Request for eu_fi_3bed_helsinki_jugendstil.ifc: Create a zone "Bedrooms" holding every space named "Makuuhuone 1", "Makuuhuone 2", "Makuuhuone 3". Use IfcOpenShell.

First a look at what the model holds.

```python
import ifcopenshell

model = ifcopenshell.open("eu_fi_3bed_helsinki_jugendstil.ifc")
print(model.schema)
seen = {}
for space in model.by_type("IfcSpace"):
    seen[space.LongName] = seen.get(space.LongName, 0) + 1
for name, count in sorted(seen.items(), key=str):
    print(count, "x", name)
print("zones:", [z.Name for z in model.by_type("IfcZone")][:20])
```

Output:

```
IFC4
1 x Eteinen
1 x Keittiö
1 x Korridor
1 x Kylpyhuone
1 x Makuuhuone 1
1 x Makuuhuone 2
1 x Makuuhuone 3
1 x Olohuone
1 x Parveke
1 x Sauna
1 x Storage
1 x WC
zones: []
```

```python
import ifcopenshell
import ifcopenshell.api.group
import ifcopenshell.api.root

model = ifcopenshell.open("eu_fi_3bed_helsinki_jugendstil.ifc")

names = {"Makuuhuone 1", "Makuuhuone 2", "Makuuhuone 3"}
spaces = [s for s in model.by_type("IfcSpace") if s.LongName in names]

zone = ifcopenshell.api.root.create_entity(model, ifc_class="IfcZone", name="Bedrooms")
ifcopenshell.api.group.assign_group(model, products=spaces, group=zone)
print(len(spaces), "spaces in", zone.Name)

model.write("eu_fi_3bed_helsinki_jugendstil_v2.ifc")
```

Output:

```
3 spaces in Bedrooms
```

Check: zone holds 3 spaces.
